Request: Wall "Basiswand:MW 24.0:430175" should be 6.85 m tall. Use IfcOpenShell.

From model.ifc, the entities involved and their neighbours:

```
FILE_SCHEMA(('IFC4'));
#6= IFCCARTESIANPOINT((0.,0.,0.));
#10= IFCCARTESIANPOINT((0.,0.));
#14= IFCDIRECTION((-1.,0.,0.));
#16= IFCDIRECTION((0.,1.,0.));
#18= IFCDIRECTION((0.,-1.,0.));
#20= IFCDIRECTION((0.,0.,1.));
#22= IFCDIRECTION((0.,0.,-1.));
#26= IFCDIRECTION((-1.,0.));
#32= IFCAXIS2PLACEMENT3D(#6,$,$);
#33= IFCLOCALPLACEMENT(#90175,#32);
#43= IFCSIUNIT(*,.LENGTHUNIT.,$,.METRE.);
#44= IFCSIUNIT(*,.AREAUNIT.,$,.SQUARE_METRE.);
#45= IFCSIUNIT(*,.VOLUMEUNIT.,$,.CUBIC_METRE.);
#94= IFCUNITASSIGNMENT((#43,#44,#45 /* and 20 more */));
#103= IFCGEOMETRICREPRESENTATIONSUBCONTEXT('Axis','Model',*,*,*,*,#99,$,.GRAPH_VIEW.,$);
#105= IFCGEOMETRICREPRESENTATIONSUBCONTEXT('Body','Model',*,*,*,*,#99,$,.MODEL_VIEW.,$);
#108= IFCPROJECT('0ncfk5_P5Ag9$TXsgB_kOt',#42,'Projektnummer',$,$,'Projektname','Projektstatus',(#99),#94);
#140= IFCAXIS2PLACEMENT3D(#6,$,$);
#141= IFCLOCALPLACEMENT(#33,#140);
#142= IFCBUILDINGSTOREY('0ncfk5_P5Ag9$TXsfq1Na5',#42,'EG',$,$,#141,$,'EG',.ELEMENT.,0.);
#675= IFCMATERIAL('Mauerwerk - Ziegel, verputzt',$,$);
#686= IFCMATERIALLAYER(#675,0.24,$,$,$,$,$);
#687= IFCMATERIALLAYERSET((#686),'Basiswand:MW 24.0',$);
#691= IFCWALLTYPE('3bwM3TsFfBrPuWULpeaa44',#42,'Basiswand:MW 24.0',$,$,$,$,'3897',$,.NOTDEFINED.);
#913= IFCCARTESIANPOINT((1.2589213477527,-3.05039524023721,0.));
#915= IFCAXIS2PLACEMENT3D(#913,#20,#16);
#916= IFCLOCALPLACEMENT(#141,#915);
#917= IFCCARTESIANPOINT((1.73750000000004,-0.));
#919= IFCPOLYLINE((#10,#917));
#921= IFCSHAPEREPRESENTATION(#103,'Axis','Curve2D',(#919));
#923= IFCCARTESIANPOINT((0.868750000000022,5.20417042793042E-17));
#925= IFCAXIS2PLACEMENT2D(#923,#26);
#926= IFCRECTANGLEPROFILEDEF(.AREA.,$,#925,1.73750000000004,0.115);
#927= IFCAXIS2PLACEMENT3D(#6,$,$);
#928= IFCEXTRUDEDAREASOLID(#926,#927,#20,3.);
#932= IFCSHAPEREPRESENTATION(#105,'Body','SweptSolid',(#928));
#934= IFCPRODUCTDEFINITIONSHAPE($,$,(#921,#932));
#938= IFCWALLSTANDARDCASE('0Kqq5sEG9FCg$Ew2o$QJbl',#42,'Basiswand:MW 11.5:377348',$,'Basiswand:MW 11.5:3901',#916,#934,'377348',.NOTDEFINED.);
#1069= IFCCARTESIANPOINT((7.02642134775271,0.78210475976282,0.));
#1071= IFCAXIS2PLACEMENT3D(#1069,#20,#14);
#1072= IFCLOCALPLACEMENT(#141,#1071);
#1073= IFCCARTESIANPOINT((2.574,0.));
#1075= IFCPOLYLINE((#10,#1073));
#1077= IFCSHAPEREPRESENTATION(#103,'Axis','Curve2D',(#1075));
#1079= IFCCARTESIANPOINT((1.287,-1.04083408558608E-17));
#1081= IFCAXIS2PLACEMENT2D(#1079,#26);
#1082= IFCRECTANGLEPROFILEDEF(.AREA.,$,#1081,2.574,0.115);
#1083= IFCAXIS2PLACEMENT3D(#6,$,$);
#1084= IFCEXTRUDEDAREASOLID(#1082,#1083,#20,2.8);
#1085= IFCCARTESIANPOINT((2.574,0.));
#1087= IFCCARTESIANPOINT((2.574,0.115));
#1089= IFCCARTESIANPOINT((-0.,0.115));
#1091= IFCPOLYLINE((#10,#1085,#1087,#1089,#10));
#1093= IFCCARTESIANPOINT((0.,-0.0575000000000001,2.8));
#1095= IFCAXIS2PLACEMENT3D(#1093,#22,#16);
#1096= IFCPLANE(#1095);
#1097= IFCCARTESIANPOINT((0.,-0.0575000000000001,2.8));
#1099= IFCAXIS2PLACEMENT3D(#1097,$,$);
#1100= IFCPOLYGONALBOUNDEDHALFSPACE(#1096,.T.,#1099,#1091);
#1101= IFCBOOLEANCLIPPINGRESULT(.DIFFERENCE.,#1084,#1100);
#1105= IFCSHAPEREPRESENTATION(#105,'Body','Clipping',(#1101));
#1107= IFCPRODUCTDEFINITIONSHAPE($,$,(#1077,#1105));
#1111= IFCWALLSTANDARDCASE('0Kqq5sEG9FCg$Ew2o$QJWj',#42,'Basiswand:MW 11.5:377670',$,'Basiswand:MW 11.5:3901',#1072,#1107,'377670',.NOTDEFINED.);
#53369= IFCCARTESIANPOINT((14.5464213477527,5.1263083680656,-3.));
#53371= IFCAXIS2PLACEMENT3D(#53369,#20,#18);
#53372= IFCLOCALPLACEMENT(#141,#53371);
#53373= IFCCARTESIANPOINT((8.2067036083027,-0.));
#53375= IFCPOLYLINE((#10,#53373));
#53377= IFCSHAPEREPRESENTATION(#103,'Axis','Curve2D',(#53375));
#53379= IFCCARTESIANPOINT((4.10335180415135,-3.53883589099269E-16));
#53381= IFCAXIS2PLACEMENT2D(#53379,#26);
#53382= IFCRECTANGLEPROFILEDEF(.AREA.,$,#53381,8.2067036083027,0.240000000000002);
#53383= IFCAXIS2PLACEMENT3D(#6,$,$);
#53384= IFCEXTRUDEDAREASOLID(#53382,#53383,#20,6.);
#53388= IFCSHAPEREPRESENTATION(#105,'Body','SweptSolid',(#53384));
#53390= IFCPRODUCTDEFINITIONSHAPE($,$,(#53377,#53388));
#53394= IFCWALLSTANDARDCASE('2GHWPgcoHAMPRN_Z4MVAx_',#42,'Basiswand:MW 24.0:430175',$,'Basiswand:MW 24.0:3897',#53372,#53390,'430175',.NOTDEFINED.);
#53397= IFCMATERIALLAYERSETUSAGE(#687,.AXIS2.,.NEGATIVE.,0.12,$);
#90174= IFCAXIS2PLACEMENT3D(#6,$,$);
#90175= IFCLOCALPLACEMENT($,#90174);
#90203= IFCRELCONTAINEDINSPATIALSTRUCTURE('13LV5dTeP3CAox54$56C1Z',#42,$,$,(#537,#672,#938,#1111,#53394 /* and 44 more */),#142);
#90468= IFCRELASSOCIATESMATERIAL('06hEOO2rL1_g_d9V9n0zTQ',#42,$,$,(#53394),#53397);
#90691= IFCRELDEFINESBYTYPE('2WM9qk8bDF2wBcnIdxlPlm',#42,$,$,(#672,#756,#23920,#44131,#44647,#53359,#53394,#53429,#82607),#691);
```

```python
import ifcopenshell
import ifcopenshell.geom
import ifcopenshell.util.representation
import ifcopenshell.util.shape
import ifcopenshell.util.unit

model = ifcopenshell.open("model.ifc")
unit_scale = ifcopenshell.util.unit.calculate_unit_scale(model)
settings = ifcopenshell.geom.settings()


def volume(element):
    """Net volume in cubic metres, openings subtracted."""
    shape = ifcopenshell.geom.create_shape(settings, element)
    return ifcopenshell.util.shape.get_volume(shape.geometry)


wall = model.by_guid("2GHWPgcoHAMPRN_Z4MVAx_")
before = volume(wall)

body = ifcopenshell.util.representation.get_representation(wall, "Model", "Body")
solid = body.Items[0]
old_height = solid.Depth
solid.Depth = 6.85 / unit_scale
after = volume(wall)

print(f"height {old_height:g} -> {solid.Depth:g}, volume {before:.3f} -> {after:.3f} m3")

model.write("model_rev.ifc")
```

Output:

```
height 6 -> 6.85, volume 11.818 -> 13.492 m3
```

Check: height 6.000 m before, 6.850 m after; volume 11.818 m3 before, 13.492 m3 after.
